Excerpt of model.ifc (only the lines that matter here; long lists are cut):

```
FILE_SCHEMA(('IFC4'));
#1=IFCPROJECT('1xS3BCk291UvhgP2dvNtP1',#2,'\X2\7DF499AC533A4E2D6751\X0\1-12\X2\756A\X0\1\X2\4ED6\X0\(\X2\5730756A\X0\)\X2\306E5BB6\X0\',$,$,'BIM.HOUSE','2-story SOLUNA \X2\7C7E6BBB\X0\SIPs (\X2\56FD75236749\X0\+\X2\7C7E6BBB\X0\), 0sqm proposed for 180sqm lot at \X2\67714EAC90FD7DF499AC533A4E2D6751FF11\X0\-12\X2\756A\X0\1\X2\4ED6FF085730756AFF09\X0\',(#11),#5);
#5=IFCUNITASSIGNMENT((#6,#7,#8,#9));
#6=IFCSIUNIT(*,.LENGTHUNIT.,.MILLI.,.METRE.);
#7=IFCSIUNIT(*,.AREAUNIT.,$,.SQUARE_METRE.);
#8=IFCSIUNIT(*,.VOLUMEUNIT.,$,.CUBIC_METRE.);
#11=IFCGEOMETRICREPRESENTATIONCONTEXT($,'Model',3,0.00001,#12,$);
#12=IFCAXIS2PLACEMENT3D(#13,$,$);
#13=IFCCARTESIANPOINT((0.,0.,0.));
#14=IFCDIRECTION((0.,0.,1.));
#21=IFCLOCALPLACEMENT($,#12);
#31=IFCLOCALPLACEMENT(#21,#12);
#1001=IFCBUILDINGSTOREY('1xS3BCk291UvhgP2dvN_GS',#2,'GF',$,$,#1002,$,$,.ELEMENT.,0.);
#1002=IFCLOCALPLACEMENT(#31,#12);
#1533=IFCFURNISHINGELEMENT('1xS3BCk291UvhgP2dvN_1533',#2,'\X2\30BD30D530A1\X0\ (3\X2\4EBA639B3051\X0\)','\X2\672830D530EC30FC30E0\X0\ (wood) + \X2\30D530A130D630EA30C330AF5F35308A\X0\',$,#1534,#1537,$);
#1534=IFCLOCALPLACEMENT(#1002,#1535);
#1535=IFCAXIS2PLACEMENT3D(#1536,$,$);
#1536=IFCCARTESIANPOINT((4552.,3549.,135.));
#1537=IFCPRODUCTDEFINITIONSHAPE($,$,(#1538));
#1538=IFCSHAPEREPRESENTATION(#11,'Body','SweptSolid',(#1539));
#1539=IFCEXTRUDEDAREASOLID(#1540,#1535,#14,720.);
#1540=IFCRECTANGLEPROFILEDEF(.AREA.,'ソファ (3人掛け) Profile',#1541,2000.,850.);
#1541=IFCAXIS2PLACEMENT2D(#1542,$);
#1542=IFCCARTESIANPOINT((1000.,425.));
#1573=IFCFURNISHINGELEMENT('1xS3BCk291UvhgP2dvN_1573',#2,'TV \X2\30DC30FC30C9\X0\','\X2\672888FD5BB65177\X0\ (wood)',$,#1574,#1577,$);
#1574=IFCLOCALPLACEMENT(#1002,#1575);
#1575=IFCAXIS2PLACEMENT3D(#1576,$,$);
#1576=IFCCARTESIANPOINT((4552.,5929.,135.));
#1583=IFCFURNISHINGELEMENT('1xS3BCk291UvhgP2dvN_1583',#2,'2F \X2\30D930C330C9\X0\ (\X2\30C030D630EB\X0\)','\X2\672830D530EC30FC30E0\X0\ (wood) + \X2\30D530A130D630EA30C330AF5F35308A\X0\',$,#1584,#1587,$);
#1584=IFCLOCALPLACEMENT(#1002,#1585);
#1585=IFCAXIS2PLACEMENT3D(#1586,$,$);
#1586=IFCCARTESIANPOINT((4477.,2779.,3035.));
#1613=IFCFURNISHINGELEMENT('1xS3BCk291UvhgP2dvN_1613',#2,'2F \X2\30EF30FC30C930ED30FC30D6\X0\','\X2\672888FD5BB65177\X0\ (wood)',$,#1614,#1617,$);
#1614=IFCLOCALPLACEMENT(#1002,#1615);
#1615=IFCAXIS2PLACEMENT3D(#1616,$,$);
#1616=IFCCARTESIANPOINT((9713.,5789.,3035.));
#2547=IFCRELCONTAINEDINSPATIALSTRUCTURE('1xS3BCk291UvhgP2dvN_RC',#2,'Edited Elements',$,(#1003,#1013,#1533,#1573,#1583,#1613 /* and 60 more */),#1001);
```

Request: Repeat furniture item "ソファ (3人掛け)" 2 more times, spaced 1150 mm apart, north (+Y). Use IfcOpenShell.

```python
import numpy as np
import ifcopenshell
import ifcopenshell.api.geometry
import ifcopenshell.api.root
import ifcopenshell.util.element
import ifcopenshell.util.placement

model = ifcopenshell.open("model.ifc")


def reuse_history(source, copy):
    """copy_class also copies each property set's owner history, people and application; keep the originals."""
    for rel in copy.IsDefinedBy:
        if rel.is_a("IfcRelDefinesByProperties") and (history := rel.RelatingPropertyDefinition.OwnerHistory):
            rel.RelatingPropertyDefinition.OwnerHistory = source.OwnerHistory
            ifcopenshell.util.element.remove_deep2(model, history)


source = model.by_guid("1xS3BCk291UvhgP2dvN_1533")
base = ifcopenshell.util.placement.get_local_placement(source.ObjectPlacement)
step = np.array([0.0, 1.0, 0.0]) * 1150.0

for i in range(1, 3):
    copy = ifcopenshell.api.root.copy_class(model, product=source)
    copy.Representation = ifcopenshell.util.element.copy_deep(
        model, source.Representation, exclude=["IfcGeometricRepresentationContext", "IfcRepresentationMap"]
    )
    reuse_history(source, copy)
    matrix = base.copy()
    matrix[:3, 3] += i * step
    print("added at", matrix[:3, 3].round(3) + 0.0)
    ifcopenshell.api.geometry.edit_object_placement(model, product=copy, matrix=matrix, is_si=False)

model.write("model-out.ifc")
```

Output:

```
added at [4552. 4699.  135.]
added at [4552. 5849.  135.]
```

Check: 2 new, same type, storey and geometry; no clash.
